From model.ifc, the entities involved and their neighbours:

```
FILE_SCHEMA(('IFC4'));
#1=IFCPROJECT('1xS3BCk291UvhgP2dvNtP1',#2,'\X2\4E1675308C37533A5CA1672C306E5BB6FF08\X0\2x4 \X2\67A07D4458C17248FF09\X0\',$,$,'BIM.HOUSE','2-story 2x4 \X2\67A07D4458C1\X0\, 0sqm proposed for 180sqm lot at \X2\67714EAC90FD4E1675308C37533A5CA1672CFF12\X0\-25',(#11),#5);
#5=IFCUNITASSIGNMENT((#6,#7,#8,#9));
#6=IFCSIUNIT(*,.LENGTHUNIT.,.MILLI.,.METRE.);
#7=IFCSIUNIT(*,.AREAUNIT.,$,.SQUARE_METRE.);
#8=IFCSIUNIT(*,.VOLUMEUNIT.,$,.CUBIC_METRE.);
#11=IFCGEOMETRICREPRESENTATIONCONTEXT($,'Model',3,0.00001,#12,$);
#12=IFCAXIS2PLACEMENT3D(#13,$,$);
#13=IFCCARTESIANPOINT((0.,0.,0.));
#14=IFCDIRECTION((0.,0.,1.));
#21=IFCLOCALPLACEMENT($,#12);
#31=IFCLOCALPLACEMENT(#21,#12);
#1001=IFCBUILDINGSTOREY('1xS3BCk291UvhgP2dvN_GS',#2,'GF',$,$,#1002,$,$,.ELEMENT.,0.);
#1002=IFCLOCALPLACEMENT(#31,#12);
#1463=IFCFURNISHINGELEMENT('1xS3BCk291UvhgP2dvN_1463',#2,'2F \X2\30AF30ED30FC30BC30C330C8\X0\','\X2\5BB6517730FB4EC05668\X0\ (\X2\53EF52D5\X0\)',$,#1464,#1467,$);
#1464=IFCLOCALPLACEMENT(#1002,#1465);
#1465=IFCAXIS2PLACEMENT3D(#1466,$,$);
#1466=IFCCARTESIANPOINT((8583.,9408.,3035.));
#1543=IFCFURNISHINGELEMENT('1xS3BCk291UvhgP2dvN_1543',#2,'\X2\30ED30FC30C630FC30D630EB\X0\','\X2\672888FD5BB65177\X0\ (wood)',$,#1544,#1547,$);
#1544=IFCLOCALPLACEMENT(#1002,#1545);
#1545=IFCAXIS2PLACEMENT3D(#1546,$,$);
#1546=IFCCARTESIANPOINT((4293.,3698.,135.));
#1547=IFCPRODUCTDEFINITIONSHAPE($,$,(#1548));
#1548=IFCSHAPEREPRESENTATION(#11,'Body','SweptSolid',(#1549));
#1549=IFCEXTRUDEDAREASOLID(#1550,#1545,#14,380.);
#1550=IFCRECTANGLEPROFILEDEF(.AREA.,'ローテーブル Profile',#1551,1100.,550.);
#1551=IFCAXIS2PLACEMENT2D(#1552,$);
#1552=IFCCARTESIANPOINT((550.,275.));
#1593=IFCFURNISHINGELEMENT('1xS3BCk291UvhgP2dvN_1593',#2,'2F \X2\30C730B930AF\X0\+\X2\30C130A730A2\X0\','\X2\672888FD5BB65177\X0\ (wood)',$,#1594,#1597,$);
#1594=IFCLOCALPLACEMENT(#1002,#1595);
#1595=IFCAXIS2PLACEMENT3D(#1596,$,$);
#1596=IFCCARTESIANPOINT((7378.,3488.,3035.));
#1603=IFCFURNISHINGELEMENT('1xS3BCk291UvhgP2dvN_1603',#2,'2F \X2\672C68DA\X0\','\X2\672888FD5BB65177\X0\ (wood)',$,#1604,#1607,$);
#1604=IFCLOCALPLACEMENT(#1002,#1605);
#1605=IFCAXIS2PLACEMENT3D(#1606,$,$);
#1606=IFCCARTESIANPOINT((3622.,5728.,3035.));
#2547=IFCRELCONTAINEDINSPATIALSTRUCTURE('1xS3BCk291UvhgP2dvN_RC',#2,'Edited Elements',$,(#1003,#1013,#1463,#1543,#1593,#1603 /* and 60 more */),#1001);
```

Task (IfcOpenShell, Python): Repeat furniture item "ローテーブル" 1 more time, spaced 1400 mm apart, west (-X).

```python
import numpy as np
import ifcopenshell
import ifcopenshell.api.geometry
import ifcopenshell.api.root
import ifcopenshell.util.element
import ifcopenshell.util.placement

model = ifcopenshell.open("model.ifc")


def reuse_history(source, copy):
    """copy_class also copies each property set's owner history, people and application; keep the originals."""
    for rel in copy.IsDefinedBy:
        if rel.is_a("IfcRelDefinesByProperties") and (history := rel.RelatingPropertyDefinition.OwnerHistory):
            rel.RelatingPropertyDefinition.OwnerHistory = source.OwnerHistory
            ifcopenshell.util.element.remove_deep2(model, history)


source = model.by_id(1543)
base = ifcopenshell.util.placement.get_local_placement(source.ObjectPlacement)
step = np.array([-1.0, 0.0, 0.0]) * 1400.0

for i in range(1, 2):
    copy = ifcopenshell.api.root.copy_class(model, product=source)
    copy.Representation = ifcopenshell.util.element.copy_deep(
        model, source.Representation, exclude=["IfcGeometricRepresentationContext", "IfcRepresentationMap"]
    )
    reuse_history(source, copy)
    matrix = base.copy()
    matrix[:3, 3] += i * step
    print("added at", matrix[:3, 3].round(3) + 0.0)
    ifcopenshell.api.geometry.edit_object_placement(model, product=copy, matrix=matrix, is_si=False)

model.write("model_edited.ifc")
```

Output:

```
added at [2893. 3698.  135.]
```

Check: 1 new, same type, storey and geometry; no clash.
